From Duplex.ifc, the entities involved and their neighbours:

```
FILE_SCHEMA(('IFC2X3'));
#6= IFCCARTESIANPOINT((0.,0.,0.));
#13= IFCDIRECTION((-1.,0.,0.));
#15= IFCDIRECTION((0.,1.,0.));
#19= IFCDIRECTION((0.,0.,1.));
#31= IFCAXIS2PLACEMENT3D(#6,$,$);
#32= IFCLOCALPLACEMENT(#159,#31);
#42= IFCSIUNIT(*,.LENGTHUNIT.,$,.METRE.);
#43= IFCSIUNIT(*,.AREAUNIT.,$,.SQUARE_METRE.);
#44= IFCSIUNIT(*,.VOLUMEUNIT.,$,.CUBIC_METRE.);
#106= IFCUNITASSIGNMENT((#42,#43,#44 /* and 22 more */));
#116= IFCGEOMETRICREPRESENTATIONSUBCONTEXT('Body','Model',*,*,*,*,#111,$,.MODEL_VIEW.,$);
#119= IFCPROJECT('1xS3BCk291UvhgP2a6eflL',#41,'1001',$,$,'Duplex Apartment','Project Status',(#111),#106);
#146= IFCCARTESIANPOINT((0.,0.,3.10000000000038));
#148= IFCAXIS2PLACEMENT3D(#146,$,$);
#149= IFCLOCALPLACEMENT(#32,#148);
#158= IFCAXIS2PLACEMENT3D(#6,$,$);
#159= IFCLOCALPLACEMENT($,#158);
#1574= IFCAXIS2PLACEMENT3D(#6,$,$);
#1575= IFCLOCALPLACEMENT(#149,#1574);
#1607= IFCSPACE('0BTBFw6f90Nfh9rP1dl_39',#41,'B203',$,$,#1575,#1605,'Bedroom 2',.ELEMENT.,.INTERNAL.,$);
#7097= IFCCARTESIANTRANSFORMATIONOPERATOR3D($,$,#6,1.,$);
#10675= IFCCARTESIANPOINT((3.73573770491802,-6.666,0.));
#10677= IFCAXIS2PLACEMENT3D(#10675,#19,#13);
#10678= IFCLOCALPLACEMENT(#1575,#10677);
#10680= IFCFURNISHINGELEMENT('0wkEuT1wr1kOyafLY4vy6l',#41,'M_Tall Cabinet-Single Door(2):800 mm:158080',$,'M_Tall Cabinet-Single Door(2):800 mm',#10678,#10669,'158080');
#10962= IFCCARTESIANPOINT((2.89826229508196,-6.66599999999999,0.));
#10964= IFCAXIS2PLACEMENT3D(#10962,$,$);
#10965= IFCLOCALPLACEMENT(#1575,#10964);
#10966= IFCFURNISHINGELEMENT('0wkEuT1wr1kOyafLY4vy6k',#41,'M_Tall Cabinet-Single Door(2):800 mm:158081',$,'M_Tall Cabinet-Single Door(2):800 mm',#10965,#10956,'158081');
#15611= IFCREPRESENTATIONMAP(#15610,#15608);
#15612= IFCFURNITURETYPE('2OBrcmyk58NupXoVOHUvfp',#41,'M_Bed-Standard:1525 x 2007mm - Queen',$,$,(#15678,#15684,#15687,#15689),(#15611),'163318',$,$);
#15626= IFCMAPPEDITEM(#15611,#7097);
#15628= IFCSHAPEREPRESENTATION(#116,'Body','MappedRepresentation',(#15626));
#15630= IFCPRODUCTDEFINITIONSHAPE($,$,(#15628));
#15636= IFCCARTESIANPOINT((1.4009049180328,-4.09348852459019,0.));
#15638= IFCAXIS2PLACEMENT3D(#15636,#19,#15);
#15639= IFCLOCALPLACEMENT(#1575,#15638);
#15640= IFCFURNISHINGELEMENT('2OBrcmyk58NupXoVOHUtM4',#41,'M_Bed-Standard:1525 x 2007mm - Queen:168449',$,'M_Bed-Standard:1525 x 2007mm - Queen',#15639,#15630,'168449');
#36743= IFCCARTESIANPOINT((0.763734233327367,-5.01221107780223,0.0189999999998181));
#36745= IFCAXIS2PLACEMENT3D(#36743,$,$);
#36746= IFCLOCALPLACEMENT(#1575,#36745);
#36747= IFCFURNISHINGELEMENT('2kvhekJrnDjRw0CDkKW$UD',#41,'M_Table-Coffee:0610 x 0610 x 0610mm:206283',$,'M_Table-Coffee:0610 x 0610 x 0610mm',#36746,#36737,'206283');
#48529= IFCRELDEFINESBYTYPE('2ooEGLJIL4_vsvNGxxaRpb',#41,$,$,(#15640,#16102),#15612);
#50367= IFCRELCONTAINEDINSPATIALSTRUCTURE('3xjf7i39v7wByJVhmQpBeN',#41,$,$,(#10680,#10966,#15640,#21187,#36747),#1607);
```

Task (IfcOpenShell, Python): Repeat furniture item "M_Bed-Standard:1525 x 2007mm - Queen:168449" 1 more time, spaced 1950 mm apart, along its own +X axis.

```python
import ifcopenshell
import ifcopenshell.api.geometry
import ifcopenshell.api.root
import ifcopenshell.util.element
import ifcopenshell.util.placement
import ifcopenshell.util.unit

model = ifcopenshell.open("Duplex.ifc")
unit_scale = ifcopenshell.util.unit.calculate_unit_scale(model)


def reuse_history(source, copy):
    """copy_class also copies each property set's owner history, people and application; keep the originals."""
    for rel in copy.IsDefinedBy:
        if rel.is_a("IfcRelDefinesByProperties") and (history := rel.RelatingPropertyDefinition.OwnerHistory):
            rel.RelatingPropertyDefinition.OwnerHistory = source.OwnerHistory
            ifcopenshell.util.element.remove_deep2(model, history)


source = model.by_guid("2OBrcmyk58NupXoVOHUtM4")
base = ifcopenshell.util.placement.get_local_placement(source.ObjectPlacement)
step = base[:3, 0] * 1.95 / unit_scale

for i in range(1, 2):
    copy = ifcopenshell.api.root.copy_class(model, product=source)
    copy.Representation = ifcopenshell.util.element.copy_deep(
        model, source.Representation, exclude=["IfcGeometricRepresentationContext", "IfcRepresentationMap"]
    )
    copy.Name = "M_Bed-Standard:1525 x 2007mm - Queen"
    copy.Tag = None
    reuse_history(source, copy)
    matrix = base.copy()
    matrix[:3, 3] += i * step
    print("added at", matrix[:3, 3].round(3) + 0.0)
    ifcopenshell.api.geometry.edit_object_placement(model, product=copy, matrix=matrix, is_si=False)

model.write("Duplex_v2.ifc")
```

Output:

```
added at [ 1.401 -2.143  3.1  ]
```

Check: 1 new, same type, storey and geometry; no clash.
